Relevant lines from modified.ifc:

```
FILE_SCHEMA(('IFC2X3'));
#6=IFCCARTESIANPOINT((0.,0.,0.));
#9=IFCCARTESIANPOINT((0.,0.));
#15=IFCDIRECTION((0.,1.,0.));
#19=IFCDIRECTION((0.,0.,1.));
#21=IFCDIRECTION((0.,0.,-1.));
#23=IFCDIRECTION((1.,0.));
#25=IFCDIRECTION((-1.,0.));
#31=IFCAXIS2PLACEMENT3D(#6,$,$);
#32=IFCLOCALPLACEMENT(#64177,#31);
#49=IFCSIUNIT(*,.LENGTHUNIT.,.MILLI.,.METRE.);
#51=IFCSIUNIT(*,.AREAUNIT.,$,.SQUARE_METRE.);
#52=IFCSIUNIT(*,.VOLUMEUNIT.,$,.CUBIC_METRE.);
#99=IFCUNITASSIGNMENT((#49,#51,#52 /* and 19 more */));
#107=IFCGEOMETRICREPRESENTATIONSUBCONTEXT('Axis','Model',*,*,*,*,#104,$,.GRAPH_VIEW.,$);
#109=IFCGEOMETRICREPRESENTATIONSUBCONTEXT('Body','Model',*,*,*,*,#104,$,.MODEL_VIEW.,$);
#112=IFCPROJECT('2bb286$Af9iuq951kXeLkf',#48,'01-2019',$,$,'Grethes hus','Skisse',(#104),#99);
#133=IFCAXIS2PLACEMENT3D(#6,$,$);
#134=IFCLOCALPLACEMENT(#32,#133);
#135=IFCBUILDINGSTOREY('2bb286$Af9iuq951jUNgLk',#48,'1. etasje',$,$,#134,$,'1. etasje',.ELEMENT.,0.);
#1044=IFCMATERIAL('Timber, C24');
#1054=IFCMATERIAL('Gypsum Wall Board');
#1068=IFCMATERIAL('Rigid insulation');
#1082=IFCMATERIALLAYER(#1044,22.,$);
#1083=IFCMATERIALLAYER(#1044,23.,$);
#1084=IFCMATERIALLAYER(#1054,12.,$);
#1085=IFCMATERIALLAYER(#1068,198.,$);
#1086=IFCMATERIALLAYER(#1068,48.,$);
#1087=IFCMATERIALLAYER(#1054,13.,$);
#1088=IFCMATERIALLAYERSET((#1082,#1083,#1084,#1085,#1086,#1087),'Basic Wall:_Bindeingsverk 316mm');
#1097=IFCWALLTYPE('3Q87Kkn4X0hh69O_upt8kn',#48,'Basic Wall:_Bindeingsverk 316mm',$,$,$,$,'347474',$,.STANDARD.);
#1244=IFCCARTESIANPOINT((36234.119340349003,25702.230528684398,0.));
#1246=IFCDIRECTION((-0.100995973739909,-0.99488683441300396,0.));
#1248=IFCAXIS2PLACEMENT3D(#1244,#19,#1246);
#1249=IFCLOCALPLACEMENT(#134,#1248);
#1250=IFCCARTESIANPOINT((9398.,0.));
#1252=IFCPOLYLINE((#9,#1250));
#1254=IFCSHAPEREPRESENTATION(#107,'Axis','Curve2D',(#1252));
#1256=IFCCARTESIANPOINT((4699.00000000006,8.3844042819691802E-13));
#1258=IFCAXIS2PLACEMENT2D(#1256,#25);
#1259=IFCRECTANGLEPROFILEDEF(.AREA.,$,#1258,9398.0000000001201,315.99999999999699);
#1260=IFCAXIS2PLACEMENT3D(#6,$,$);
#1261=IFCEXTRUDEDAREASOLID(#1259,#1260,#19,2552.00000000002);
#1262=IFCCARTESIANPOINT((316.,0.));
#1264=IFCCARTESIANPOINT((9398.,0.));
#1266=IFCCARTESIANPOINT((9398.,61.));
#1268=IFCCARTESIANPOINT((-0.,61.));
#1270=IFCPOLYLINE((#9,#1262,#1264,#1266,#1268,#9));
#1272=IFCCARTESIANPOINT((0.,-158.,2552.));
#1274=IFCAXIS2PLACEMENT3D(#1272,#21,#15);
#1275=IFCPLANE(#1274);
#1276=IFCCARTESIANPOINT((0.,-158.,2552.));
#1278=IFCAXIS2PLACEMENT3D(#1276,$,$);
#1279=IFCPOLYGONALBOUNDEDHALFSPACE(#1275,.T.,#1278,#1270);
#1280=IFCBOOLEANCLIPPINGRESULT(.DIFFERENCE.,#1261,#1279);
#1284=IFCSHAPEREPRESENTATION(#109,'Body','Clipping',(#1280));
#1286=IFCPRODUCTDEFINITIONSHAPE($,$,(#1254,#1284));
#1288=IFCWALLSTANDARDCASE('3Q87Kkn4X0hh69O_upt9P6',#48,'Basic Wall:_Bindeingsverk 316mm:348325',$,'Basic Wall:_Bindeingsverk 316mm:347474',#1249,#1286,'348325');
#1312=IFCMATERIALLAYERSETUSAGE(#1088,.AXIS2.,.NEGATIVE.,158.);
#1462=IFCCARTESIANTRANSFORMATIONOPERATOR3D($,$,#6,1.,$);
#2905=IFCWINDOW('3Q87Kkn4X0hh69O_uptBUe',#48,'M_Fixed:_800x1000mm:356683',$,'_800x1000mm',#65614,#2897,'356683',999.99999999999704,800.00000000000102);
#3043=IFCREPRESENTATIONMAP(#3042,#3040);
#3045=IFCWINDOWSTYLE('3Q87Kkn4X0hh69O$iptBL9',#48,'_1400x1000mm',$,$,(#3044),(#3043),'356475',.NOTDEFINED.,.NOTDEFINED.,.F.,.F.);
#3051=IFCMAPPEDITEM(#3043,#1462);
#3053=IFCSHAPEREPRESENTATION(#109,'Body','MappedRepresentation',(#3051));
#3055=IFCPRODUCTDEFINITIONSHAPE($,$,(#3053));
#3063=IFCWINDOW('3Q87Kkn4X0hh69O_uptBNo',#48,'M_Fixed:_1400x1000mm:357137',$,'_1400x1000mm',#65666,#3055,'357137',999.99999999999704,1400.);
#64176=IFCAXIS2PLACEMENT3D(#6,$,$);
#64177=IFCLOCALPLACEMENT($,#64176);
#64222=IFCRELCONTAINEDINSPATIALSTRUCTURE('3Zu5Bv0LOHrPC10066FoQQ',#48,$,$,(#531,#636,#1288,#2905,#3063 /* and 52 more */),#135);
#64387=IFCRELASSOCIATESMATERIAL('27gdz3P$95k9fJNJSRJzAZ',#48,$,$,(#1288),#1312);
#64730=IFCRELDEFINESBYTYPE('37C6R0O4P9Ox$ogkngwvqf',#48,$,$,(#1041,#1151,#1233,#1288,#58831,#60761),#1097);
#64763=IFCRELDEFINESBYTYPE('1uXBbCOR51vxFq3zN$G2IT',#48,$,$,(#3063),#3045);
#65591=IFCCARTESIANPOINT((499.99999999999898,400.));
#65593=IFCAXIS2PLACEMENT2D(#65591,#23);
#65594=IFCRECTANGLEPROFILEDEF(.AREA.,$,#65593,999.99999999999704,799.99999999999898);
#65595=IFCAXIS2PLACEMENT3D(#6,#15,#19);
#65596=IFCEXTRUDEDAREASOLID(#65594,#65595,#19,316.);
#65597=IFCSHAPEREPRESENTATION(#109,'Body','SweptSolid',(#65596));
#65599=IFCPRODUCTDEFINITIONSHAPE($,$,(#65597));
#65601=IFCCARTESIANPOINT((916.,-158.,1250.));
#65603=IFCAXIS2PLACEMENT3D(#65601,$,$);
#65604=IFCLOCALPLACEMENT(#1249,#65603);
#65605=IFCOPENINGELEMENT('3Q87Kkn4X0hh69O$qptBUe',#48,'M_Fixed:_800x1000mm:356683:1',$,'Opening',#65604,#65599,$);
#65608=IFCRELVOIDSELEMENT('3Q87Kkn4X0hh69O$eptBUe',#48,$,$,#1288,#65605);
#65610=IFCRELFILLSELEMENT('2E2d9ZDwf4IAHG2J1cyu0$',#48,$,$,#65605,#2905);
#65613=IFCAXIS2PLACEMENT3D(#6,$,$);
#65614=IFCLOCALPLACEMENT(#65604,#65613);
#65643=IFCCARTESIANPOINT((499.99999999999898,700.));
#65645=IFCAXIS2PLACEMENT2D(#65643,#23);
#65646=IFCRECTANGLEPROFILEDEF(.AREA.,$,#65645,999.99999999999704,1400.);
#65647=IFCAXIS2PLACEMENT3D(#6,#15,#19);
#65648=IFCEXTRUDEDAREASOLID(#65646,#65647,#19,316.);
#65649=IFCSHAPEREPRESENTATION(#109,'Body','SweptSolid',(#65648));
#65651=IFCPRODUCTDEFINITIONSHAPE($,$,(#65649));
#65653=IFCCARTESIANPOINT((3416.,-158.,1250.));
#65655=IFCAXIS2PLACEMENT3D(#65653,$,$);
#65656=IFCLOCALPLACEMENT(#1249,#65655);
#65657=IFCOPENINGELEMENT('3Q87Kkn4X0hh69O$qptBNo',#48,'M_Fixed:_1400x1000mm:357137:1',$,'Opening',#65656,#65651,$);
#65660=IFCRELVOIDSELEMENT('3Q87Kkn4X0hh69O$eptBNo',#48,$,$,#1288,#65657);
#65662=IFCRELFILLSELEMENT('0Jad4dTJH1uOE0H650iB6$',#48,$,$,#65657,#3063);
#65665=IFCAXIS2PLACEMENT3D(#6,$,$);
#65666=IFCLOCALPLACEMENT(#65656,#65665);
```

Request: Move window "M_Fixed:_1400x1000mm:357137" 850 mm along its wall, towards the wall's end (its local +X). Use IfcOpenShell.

```python
import ifcopenshell
import ifcopenshell.api.geometry
import ifcopenshell.util.placement
import ifcopenshell.util.unit

model = ifcopenshell.open("modified.ifc")
unit_scale = ifcopenshell.util.unit.calculate_unit_scale(model)

window = model.by_guid("3Q87Kkn4X0hh69O_uptBNo")
opening = window.FillsVoids[0].RelatingOpeningElement
wall = opening.VoidsElements[0].RelatingBuildingElement

wall_matrix = ifcopenshell.util.placement.get_local_placement(wall.ObjectPlacement)
shift = wall_matrix[:3, 0] * 0.85 / unit_scale
before = ifcopenshell.util.placement.get_local_placement(window.ObjectPlacement)[:3, 3].copy()

# The window is placed relative to its opening, so it follows when the opening moves.
matrix = ifcopenshell.util.placement.get_local_placement(opening.ObjectPlacement)
matrix[:3, 3] += shift
ifcopenshell.api.geometry.edit_object_placement(
    model, product=opening, matrix=matrix, is_si=False, should_transform_children=True
)

after = ifcopenshell.util.placement.get_local_placement(window.ObjectPlacement)[:3, 3]
print("window moved by", (after - before).round(3) + 0.0)

model.write("modified-out.ifc")
```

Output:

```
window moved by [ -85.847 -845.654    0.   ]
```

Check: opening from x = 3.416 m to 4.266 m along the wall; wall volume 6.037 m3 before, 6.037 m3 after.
